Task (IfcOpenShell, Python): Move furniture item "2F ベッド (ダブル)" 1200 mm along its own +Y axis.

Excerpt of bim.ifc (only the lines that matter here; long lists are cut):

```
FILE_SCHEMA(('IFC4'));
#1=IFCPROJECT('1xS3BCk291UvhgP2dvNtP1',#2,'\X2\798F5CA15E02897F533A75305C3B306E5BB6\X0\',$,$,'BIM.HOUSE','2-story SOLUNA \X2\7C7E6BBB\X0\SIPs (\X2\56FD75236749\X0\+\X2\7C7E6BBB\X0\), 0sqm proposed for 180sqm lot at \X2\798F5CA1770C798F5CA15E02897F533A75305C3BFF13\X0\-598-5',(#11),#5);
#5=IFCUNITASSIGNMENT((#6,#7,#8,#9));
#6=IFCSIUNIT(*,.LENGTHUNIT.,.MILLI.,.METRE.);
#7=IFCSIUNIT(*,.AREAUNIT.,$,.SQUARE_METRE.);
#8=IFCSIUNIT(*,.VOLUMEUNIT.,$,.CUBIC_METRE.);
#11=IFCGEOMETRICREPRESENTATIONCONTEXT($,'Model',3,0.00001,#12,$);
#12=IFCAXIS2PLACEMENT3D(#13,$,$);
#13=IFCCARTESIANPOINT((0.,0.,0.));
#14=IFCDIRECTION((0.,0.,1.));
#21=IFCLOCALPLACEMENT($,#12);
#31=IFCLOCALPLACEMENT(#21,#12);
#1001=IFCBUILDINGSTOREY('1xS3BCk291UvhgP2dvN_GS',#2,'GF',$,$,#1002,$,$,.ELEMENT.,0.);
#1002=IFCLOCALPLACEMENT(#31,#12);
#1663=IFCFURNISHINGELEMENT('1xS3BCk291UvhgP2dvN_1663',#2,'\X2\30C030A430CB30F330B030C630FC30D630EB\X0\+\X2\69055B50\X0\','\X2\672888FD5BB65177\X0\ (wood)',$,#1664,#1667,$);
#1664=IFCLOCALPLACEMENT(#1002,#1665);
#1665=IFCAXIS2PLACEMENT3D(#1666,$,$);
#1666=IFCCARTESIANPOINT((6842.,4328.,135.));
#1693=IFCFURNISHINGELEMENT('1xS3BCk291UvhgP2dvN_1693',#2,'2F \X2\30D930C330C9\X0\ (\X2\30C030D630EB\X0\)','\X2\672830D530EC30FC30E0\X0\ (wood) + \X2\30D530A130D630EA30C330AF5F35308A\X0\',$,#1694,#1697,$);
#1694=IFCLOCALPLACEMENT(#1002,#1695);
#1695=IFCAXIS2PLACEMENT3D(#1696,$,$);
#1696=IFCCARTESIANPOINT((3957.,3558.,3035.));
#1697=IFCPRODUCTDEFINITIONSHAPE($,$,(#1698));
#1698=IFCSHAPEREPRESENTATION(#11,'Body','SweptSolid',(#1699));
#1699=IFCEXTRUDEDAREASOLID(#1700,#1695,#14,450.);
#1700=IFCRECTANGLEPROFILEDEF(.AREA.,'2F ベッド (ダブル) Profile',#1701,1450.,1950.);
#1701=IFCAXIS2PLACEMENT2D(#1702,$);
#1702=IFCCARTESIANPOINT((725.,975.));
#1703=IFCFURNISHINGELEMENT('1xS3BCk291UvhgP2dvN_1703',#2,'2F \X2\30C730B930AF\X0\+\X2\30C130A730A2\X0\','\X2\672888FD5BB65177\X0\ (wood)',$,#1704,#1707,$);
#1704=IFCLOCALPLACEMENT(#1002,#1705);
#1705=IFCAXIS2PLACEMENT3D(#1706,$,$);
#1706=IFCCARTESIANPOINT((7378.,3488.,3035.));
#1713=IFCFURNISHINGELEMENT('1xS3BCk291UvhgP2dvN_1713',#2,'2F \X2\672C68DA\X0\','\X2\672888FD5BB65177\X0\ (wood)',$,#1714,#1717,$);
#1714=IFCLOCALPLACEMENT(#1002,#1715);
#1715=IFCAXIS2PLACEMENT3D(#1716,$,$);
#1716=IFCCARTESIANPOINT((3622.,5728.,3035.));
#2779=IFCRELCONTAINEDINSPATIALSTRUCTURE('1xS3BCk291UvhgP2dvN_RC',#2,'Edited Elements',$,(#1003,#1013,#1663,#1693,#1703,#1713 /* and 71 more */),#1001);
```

```python
import ifcopenshell
import ifcopenshell.api.geometry
import ifcopenshell.util.placement
import ifcopenshell.util.unit

model = ifcopenshell.open("bim.ifc")
unit_scale = ifcopenshell.util.unit.calculate_unit_scale(model)

item = model.by_guid("1xS3BCk291UvhgP2dvN_1693")
matrix = ifcopenshell.util.placement.get_local_placement(item.ObjectPlacement)
matrix[:3, 3] += matrix[:3, 1] * 1.2 / unit_scale
ifcopenshell.api.geometry.edit_object_placement(model, product=item, matrix=matrix, is_si=False)

print(ifcopenshell.util.placement.get_local_placement(item.ObjectPlacement).round(3) + 0.0)

model.write("bim_updated.ifc")
```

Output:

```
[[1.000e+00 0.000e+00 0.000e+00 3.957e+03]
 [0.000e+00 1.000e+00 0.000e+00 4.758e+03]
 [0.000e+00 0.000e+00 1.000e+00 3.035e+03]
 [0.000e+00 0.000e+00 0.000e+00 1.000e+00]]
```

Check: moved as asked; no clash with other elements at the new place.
